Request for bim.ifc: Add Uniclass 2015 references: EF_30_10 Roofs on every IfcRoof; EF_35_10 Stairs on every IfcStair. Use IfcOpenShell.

First a look at what the model holds.

```python
import ifcopenshell

model = ifcopenshell.open("bim.ifc")
print(model.schema)
print("classifications:", [c.Name for c in model.by_type("IfcClassification")])
for ifc_class in ("IfcDoor", "IfcRoof", "IfcStair", "IfcWall", "IfcWindow"):
    print(ifc_class, len(model.by_type(ifc_class)))
```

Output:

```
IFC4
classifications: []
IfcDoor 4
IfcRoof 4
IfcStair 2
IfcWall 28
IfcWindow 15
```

```python
import ifcopenshell
import ifcopenshell.api.classification

model = ifcopenshell.open("bim.ifc")

system = ifcopenshell.api.classification.add_classification(model, classification="Uniclass 2015")

codes = {
    "IfcRoof": ("EF_30_10", "Roofs"),
    "IfcStair": ("EF_35_10", "Stairs"),
}
for ifc_class, (code, name) in codes.items():
    products = model.by_type(ifc_class)
    ifcopenshell.api.classification.add_reference(
        model, products=products, classification=system, identification=code, name=name
    )
    print(code, len(products))

model.write("bim_rev.ifc")
```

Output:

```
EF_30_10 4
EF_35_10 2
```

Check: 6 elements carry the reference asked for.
